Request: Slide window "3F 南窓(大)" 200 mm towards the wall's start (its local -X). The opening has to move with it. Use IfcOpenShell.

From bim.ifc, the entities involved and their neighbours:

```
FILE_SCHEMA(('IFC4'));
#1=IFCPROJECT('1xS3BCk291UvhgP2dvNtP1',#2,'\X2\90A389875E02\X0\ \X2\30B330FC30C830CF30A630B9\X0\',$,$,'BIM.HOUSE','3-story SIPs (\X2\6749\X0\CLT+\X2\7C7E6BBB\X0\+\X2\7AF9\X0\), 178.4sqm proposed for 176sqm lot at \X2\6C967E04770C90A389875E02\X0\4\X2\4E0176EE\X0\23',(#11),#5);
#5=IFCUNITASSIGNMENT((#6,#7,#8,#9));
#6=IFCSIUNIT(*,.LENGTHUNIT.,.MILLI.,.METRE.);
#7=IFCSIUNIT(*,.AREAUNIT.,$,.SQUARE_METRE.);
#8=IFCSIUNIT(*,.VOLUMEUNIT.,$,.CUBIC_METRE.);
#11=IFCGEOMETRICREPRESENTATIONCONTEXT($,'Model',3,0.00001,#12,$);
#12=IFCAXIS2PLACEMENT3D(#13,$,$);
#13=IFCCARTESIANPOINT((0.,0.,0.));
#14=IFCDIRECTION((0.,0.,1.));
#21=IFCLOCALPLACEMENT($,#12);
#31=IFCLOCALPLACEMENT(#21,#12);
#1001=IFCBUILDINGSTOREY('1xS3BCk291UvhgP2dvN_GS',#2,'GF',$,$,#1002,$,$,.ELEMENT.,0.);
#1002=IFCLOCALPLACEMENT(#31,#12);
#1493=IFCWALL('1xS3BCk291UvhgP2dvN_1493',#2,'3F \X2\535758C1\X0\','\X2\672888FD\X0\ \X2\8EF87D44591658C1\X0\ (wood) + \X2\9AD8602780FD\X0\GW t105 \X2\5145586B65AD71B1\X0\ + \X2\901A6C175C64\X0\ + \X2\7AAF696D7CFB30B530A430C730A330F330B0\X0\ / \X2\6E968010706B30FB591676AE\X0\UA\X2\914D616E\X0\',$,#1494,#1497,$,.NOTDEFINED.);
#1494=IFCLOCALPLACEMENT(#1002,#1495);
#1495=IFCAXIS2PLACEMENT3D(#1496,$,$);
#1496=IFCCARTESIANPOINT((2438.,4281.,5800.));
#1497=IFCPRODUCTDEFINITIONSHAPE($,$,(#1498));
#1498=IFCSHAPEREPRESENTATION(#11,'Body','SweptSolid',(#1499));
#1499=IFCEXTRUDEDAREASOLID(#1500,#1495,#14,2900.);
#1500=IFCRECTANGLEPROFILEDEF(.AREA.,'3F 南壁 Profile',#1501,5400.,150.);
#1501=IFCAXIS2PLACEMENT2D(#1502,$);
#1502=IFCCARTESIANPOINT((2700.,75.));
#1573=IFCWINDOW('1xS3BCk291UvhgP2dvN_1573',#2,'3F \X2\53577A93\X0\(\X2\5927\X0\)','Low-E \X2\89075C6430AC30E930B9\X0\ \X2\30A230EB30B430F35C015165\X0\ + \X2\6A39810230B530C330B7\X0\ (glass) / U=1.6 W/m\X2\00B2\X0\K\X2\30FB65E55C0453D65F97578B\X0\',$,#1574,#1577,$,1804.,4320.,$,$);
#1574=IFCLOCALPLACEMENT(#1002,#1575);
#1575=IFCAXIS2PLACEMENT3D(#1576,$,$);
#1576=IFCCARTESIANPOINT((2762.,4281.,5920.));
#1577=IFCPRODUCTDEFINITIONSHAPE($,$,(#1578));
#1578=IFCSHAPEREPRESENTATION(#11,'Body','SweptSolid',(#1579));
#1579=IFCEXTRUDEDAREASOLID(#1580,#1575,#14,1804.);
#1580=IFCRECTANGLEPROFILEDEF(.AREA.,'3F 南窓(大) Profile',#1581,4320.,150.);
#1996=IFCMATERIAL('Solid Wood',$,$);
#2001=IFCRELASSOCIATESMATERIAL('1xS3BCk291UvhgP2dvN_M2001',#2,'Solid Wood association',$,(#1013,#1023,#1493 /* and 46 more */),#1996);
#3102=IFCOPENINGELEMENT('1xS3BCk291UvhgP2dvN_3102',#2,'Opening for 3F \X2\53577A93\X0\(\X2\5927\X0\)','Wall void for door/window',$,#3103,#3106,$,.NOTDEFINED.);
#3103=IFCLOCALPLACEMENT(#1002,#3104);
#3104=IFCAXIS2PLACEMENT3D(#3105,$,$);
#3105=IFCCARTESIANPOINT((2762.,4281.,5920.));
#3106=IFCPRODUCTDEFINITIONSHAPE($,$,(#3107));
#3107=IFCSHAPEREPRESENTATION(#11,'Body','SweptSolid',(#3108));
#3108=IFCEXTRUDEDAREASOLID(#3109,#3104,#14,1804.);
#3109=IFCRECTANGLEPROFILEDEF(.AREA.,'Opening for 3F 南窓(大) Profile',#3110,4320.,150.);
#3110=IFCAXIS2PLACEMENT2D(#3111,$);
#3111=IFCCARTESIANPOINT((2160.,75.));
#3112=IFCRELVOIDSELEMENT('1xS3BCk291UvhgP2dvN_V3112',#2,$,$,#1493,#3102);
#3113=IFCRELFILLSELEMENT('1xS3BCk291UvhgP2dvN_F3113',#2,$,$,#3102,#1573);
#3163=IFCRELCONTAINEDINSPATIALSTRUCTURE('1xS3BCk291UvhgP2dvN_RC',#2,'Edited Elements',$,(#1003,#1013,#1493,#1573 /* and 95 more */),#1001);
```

```python
import ifcopenshell
import ifcopenshell.api.geometry
import ifcopenshell.util.placement

model = ifcopenshell.open("bim.ifc")

window = model.by_guid("1xS3BCk291UvhgP2dvN_1573")
opening = window.FillsVoids[0].RelatingOpeningElement
wall = opening.VoidsElements[0].RelatingBuildingElement

wall_matrix = ifcopenshell.util.placement.get_local_placement(wall.ObjectPlacement)
shift = wall_matrix[:3, 0] * -200.0
before = ifcopenshell.util.placement.get_local_placement(window.ObjectPlacement)[:3, 3].copy()

# The window is not placed relative to its opening, so move both.
for product in (opening, window):
    matrix = ifcopenshell.util.placement.get_local_placement(product.ObjectPlacement)
    matrix[:3, 3] += shift
    ifcopenshell.api.geometry.edit_object_placement(model, product=product, matrix=matrix, is_si=False)

after = ifcopenshell.util.placement.get_local_placement(window.ObjectPlacement)[:3, 3]
print("window moved by", (after - before).round(3) + 0.0)

model.write("bim_rev.ifc")
```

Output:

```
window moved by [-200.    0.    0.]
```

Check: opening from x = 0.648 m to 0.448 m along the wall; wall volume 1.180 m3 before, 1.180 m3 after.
